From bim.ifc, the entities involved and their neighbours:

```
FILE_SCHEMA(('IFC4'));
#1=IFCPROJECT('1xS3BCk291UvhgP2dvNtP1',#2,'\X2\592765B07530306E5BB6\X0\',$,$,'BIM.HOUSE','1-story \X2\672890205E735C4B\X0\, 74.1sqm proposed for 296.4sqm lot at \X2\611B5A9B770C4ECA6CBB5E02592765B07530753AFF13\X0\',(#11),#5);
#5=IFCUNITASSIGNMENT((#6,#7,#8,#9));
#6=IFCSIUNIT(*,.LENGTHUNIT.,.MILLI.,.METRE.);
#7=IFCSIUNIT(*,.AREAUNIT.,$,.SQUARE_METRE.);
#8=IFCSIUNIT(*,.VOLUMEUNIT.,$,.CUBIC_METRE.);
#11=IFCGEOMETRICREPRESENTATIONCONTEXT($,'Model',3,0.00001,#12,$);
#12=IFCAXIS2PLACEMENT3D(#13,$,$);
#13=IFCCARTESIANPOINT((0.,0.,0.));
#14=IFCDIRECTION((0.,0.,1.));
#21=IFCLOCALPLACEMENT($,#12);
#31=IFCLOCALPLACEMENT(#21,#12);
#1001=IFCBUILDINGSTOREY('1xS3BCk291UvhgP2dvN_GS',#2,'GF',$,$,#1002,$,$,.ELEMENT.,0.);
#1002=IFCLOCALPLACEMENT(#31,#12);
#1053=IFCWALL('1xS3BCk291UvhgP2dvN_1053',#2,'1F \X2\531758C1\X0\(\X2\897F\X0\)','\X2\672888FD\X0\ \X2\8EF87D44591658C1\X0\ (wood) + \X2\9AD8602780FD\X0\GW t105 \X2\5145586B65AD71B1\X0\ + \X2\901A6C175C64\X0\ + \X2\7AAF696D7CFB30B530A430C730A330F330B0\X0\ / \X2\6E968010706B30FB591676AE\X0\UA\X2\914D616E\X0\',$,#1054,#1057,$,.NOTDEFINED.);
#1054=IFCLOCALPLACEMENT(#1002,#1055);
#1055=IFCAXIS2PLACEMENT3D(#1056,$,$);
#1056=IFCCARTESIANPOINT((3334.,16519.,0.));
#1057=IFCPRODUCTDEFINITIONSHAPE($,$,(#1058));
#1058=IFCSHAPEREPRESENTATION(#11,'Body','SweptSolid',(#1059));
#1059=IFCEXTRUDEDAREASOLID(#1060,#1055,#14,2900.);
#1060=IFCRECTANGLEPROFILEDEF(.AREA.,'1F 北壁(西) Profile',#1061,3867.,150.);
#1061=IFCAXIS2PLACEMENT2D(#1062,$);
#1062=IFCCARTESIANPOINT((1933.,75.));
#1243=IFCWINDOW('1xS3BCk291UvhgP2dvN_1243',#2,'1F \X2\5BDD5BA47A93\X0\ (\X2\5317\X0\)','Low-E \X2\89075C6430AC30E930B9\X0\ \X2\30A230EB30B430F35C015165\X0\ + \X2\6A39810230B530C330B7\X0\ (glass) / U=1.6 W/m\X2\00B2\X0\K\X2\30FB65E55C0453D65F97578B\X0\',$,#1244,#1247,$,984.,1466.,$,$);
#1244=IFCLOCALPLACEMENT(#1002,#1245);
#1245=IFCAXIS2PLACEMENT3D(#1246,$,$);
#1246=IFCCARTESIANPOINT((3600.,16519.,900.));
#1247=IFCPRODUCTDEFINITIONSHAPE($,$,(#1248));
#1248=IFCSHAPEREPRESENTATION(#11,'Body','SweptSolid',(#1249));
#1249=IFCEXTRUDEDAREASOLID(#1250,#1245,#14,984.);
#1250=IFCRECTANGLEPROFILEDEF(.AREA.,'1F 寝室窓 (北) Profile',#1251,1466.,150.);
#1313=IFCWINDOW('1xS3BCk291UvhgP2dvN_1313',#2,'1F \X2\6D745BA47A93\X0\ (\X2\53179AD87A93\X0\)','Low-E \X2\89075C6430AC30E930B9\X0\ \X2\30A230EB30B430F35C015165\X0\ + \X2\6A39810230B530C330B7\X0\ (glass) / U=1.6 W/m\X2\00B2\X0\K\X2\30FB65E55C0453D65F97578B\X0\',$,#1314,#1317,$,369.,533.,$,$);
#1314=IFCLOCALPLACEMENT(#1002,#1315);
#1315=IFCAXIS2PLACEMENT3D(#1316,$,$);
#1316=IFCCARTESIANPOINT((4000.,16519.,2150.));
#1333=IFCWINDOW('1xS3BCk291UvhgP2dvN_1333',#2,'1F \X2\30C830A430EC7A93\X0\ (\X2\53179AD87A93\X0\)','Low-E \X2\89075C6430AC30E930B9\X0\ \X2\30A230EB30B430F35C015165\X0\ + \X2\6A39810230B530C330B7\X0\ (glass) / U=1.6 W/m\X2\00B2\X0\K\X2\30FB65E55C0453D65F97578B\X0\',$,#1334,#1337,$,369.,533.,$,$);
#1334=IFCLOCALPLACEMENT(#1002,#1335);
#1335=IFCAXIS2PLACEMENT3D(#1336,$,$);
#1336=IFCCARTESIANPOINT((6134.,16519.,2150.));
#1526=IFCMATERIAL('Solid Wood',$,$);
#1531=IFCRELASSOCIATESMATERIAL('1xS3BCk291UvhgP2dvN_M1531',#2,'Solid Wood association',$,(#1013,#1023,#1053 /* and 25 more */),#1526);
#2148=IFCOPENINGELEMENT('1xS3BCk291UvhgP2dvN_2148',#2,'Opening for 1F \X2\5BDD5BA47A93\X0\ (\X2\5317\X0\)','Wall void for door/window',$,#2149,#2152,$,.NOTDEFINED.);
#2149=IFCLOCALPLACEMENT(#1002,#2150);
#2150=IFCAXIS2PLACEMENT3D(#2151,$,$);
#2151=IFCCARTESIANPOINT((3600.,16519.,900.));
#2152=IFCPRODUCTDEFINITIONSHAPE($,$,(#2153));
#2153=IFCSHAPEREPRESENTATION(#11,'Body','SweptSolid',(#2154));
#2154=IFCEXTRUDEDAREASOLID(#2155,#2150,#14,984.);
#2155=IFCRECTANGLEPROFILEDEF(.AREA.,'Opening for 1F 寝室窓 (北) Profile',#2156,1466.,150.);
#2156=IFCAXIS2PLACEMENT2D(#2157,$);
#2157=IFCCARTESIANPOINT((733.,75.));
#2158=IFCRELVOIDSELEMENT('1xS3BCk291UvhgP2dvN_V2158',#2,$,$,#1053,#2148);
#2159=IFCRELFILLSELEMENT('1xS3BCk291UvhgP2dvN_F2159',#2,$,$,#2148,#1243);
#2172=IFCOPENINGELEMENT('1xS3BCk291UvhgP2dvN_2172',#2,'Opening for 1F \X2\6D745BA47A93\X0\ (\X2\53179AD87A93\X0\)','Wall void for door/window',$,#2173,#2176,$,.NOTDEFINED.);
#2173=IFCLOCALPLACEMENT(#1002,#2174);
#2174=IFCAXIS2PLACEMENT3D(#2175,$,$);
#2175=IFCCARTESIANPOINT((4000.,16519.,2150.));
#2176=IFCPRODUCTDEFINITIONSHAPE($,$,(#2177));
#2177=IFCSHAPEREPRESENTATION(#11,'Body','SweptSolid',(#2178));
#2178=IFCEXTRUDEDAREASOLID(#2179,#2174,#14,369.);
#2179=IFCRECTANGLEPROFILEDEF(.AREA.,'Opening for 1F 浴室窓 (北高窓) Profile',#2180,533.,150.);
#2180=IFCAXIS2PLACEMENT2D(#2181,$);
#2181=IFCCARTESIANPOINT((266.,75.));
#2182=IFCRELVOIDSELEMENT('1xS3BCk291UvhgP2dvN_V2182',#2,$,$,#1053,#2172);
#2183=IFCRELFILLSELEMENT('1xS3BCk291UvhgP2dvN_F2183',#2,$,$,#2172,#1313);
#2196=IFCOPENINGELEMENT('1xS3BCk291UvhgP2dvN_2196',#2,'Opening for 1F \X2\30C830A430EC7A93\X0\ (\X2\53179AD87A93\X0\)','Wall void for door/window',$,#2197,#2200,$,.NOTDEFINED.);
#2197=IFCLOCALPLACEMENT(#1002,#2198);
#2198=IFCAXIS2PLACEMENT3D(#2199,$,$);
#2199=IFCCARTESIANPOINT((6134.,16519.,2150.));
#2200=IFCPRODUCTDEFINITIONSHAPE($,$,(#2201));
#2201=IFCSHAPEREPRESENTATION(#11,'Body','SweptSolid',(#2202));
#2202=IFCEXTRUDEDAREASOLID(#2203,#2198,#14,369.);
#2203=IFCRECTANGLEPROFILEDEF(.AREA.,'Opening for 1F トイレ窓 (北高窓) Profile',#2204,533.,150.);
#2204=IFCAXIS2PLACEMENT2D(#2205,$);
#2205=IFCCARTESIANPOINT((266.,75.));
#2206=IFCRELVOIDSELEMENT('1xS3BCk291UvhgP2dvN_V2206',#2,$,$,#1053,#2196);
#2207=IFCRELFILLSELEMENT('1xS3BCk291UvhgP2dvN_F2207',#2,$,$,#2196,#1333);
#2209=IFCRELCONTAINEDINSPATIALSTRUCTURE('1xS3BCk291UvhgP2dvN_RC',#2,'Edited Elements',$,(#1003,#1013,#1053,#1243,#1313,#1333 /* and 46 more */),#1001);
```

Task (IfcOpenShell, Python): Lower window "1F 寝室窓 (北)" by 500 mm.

```python
import numpy as np
import ifcopenshell
import ifcopenshell.api.geometry
import ifcopenshell.util.placement
import ifcopenshell.util.unit

model = ifcopenshell.open("bim.ifc")
unit_scale = ifcopenshell.util.unit.calculate_unit_scale(model)

window = model.by_guid("1xS3BCk291UvhgP2dvN_1243")
opening = window.FillsVoids[0].RelatingOpeningElement
dz = -0.5 / unit_scale

shift = np.array([0.0, 0.0, dz])
# The window is not placed relative to its opening, so move both.
for product in (opening, window):
    matrix = ifcopenshell.util.placement.get_local_placement(product.ObjectPlacement)
    matrix[:3, 3] += shift
    ifcopenshell.api.geometry.edit_object_placement(model, product=product, matrix=matrix, is_si=False)

print(f"moved by {dz * unit_scale:+.3f} m")

model.write("bim_edited.ifc")
```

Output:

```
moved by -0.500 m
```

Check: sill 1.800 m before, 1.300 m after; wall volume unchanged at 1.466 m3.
